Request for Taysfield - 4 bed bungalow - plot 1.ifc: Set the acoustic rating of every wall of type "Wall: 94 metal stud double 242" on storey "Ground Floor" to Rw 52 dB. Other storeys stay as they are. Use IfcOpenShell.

First a look at what the model holds.

```python
import ifcopenshell
import ifcopenshell.util.element

model = ifcopenshell.open("Taysfield - 4 bed bungalow - plot 1.ifc")
print(model.schema)
storey = next(s for s in model.by_type("IfcBuildingStorey") if s.Name == "Ground Floor")
walls = [e for e in ifcopenshell.util.element.get_decomposition(storey) if e.is_a("IfcWall")]
seen = {}
for e in walls:
    element_type = ifcopenshell.util.element.get_type(e)
    key = (element_type.Name if element_type != e and element_type else None, ifcopenshell.util.element.get_pset(e, "Pset_WallCommon", "AcousticRating"))
    seen[key] = seen.get(key, 0) + 1
for (name, value), count in sorted(seen.items(), key=str):
    print(count, "x", name, "|", value)
```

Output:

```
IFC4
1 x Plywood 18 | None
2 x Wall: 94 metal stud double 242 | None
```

```python
import ifcopenshell
import ifcopenshell.api.pset
import ifcopenshell.util.element

model = ifcopenshell.open("Taysfield - 4 bed bungalow - plot 1.ifc")

storey = next(s for s in model.by_type("IfcBuildingStorey") if s.Name == "Ground Floor")
walls = [e for e in ifcopenshell.util.element.get_decomposition(storey) if e.is_a("IfcWall")]

count = 0
for e in walls:
    element_type = ifcopenshell.util.element.get_type(e)
    if element_type in (None, e) or element_type.Name != "Wall: 94 metal stud double 242":
        continue
    # add_pset returns the element's existing set when there is one.
    pset = ifcopenshell.api.pset.add_pset(model, product=e, name="Pset_WallCommon")
    ifcopenshell.api.pset.edit_pset(model, pset=pset, properties={"AcousticRating": "Rw 52 dB"})
    count += 1

print(count, "walls updated")

model.write("Taysfield - 4 bed bungalow - plot 1_v2.ifc")
```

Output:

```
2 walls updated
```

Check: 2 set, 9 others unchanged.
